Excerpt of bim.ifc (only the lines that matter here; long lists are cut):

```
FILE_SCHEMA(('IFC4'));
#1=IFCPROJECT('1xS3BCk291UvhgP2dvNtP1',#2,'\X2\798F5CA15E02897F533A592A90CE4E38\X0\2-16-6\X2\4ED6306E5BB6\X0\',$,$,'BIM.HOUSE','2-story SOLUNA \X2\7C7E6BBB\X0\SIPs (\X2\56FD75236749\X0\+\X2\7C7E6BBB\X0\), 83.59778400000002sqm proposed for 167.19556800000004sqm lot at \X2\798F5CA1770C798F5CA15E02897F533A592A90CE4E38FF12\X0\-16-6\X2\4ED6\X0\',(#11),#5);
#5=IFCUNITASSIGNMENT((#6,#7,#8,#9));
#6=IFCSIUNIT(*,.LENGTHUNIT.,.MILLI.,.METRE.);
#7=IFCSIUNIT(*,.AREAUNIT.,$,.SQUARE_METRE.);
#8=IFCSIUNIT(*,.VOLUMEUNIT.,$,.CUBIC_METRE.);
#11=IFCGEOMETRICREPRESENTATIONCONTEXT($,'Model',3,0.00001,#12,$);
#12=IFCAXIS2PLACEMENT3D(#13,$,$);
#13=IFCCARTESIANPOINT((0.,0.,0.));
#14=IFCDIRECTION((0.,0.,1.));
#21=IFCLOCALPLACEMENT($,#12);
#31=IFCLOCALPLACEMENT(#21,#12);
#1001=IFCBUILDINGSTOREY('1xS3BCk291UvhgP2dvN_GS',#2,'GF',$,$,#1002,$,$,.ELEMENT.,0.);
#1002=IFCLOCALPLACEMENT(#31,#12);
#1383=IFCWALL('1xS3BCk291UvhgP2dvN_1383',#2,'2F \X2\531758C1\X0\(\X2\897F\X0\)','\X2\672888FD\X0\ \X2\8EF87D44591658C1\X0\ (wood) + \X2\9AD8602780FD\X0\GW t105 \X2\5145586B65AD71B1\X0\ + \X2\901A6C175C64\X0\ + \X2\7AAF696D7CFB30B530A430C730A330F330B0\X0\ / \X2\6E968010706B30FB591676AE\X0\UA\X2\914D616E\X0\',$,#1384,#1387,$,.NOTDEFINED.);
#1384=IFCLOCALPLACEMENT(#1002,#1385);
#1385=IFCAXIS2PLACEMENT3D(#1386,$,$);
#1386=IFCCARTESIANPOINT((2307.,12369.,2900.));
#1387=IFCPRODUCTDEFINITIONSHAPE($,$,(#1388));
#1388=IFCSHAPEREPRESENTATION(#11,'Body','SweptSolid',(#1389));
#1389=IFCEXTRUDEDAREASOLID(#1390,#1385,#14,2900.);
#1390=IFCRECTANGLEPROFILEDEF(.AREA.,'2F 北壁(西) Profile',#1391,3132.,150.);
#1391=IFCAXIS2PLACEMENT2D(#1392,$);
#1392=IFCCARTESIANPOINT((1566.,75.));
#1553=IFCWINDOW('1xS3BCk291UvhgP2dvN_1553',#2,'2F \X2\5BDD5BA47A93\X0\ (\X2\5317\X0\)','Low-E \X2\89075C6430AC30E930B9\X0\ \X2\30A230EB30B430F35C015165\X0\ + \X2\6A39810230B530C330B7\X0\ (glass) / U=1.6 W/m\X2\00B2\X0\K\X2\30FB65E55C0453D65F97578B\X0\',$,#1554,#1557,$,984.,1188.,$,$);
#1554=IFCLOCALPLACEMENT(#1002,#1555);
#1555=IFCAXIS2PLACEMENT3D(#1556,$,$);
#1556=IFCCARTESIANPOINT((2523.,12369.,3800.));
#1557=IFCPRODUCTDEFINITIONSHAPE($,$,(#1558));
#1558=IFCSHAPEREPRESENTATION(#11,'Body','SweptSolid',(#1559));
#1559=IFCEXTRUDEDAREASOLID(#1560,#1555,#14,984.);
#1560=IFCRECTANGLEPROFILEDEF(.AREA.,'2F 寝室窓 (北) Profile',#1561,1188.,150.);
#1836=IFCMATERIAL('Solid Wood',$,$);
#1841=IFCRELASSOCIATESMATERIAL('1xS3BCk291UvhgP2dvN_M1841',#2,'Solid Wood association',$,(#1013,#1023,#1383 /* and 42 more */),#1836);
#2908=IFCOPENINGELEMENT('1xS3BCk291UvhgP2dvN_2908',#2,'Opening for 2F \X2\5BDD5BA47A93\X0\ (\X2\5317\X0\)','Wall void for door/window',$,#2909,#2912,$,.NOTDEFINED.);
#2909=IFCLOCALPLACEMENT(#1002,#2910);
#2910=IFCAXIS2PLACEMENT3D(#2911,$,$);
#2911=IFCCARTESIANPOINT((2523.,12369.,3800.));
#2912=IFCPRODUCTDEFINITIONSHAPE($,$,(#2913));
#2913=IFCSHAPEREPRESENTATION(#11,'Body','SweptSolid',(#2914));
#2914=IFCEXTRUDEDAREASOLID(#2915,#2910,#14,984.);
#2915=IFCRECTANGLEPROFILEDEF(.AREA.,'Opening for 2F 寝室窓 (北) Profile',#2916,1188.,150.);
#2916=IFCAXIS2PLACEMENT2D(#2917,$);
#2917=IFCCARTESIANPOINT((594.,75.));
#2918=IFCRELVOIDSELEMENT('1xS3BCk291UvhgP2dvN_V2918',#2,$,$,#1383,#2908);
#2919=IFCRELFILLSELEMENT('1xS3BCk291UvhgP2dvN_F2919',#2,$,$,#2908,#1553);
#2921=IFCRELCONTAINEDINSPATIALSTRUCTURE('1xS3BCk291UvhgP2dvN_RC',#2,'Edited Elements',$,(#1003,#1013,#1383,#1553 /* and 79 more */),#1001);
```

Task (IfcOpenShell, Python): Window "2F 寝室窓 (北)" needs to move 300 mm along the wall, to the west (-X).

```python
import ifcopenshell
import ifcopenshell.api.geometry
import ifcopenshell.util.placement

model = ifcopenshell.open("bim.ifc")

window = model.by_id(1553)
opening = window.FillsVoids[0].RelatingOpeningElement
wall = opening.VoidsElements[0].RelatingBuildingElement

wall_matrix = ifcopenshell.util.placement.get_local_placement(wall.ObjectPlacement)
shift = wall_matrix[:3, 0] * -300.0
before = ifcopenshell.util.placement.get_local_placement(window.ObjectPlacement)[:3, 3].copy()

# The window is not placed relative to its opening, so move both.
for product in (opening, window):
    matrix = ifcopenshell.util.placement.get_local_placement(product.ObjectPlacement)
    matrix[:3, 3] += shift
    ifcopenshell.api.geometry.edit_object_placement(model, product=product, matrix=matrix, is_si=False)

after = ifcopenshell.util.placement.get_local_placement(window.ObjectPlacement)[:3, 3]
print("window moved by", (after - before).round(3) + 0.0)

model.write("bim_rev.ifc")
```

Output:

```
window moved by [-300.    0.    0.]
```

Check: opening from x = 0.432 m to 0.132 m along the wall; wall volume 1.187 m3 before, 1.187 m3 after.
